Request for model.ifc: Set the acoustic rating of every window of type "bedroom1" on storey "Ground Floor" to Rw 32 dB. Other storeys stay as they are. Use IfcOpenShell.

First a look at what the model holds.

```python
import ifcopenshell
import ifcopenshell.util.element

model = ifcopenshell.open("model.ifc")
print(model.schema)
storey = next(s for s in model.by_type("IfcBuildingStorey") if s.Name == "Ground Floor")
windows = [e for e in ifcopenshell.util.element.get_decomposition(storey) if e.is_a("IfcWindow")]
seen = {}
for e in windows:
    element_type = ifcopenshell.util.element.get_type(e)
    key = (element_type.Name if element_type != e and element_type else None, ifcopenshell.util.element.get_pset(e, "Pset_WindowCommon", "AcousticRating"))
    seen[key] = seen.get(key, 0) + 1
for (name, value), count in sorted(seen.items(), key=str):
    print(count, "x", name, "|", value)
```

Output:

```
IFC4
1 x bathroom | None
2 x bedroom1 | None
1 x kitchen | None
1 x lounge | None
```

```python
import ifcopenshell
import ifcopenshell.api.pset
import ifcopenshell.util.element

model = ifcopenshell.open("model.ifc")

storey = next(s for s in model.by_type("IfcBuildingStorey") if s.Name == "Ground Floor")
windows = [e for e in ifcopenshell.util.element.get_decomposition(storey) if e.is_a("IfcWindow")]

count = 0
for e in windows:
    element_type = ifcopenshell.util.element.get_type(e)
    if element_type in (None, e) or element_type.Name != "bedroom1":
        continue
    # add_pset returns the element's existing set when there is one.
    pset = ifcopenshell.api.pset.add_pset(model, product=e, name="Pset_WindowCommon")
    ifcopenshell.api.pset.edit_pset(model, pset=pset, properties={"AcousticRating": "Rw 32 dB"})
    count += 1

print(count, "windows updated")

model.write("model_rev.ifc")
```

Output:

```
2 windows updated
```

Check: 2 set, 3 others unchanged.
